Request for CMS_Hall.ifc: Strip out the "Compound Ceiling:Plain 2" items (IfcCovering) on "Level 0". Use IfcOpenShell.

First a look at what the model holds.

```python
import ifcopenshell
import ifcopenshell.util.element

model = ifcopenshell.open("CMS_Hall.ifc")
print(model.schema)
storey = next(s for s in model.by_type("IfcBuildingStorey") if s.Name == "Level 0")
coverings = [e for e in ifcopenshell.util.element.get_decomposition(storey) if e.is_a("IfcCovering")]
seen = {}
for e in coverings:
    element_type = ifcopenshell.util.element.get_type(e)
    name = element_type.Name if element_type not in (None, e) else None
    seen[name] = seen.get(name, 0) + 1
for name, count in sorted(seen.items(), key=str):
    print(count, "x", name)
```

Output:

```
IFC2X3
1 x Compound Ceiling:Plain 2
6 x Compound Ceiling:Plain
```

```python
import ifcopenshell
import ifcopenshell.api.root
import ifcopenshell.util.element

model = ifcopenshell.open("CMS_Hall.ifc")

storey = next(s for s in model.by_type("IfcBuildingStorey") if s.Name == "Level 0")
coverings = [e for e in ifcopenshell.util.element.get_decomposition(storey) if e.is_a("IfcCovering")]
targets = [e for e in coverings if (t := ifcopenshell.util.element.get_type(e)) not in (None, e) and t.Name == "Compound Ceiling:Plain 2"]

for e in targets:
    ifcopenshell.api.root.remove_product(model, product=e)
print(len(targets), "removed")

model.write("CMS_Hall_edited.ifc")
```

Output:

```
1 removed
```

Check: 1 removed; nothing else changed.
